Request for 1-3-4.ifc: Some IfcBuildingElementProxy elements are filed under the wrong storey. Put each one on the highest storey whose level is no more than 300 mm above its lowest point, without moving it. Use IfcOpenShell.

First a look at what the model holds.

```python
import ifcopenshell
import ifcopenshell.util.element
import ifcopenshell.util.placement

model = ifcopenshell.open("1-3-4.ifc")
print(model.schema)
for storey in model.by_type("IfcBuildingStorey"):
    level = ifcopenshell.util.placement.get_storey_elevation(storey)
    count = sum(e.is_a("IfcBuildingElementProxy") for e in ifcopenshell.util.element.get_contained(storey))
    print(storey.id(), storey.Name, round(level, 3), count, sep=" | ")
```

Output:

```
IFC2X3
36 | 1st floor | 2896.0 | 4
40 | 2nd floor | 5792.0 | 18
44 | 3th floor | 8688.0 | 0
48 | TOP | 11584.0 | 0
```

```python
import ifcopenshell
import ifcopenshell.api.spatial
import ifcopenshell.geom
import ifcopenshell.util.element
import ifcopenshell.util.placement
import ifcopenshell.util.shape
import ifcopenshell.util.unit

model = ifcopenshell.open("1-3-4.ifc")
unit_scale = ifcopenshell.util.unit.calculate_unit_scale(model)
settings = ifcopenshell.geom.settings()

levels = sorted(
    ((ifcopenshell.util.placement.get_storey_elevation(s) * unit_scale, s) for s in model.by_type("IfcBuildingStorey")),
    key=lambda pair: pair[0],
)

for e in model.by_type("IfcBuildingElementProxy"):
    current = e.ContainedInStructure[0].RelatingStructure if e.ContainedInStructure else None
    if current is None or not current.is_a("IfcBuildingStorey"):
        continue
    shape = ifcopenshell.geom.create_shape(settings, e)
    bottom = ifcopenshell.util.shape.get_shape_bottom_elevation(shape, shape.geometry)
    below = [s for level, s in levels if level <= bottom + 0.3]
    storey = below[-1] if below else levels[0][1]
    if storey != current:
        # assign_container keeps the world position.
        ifcopenshell.api.spatial.assign_container(model, products=[e], relating_structure=storey)
        print(e.id(), current.Name, "->", storey.Name)

model.write("1-3-4_edited.ifc")
```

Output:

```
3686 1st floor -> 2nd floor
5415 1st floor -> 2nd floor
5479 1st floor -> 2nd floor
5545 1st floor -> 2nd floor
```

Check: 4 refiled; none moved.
